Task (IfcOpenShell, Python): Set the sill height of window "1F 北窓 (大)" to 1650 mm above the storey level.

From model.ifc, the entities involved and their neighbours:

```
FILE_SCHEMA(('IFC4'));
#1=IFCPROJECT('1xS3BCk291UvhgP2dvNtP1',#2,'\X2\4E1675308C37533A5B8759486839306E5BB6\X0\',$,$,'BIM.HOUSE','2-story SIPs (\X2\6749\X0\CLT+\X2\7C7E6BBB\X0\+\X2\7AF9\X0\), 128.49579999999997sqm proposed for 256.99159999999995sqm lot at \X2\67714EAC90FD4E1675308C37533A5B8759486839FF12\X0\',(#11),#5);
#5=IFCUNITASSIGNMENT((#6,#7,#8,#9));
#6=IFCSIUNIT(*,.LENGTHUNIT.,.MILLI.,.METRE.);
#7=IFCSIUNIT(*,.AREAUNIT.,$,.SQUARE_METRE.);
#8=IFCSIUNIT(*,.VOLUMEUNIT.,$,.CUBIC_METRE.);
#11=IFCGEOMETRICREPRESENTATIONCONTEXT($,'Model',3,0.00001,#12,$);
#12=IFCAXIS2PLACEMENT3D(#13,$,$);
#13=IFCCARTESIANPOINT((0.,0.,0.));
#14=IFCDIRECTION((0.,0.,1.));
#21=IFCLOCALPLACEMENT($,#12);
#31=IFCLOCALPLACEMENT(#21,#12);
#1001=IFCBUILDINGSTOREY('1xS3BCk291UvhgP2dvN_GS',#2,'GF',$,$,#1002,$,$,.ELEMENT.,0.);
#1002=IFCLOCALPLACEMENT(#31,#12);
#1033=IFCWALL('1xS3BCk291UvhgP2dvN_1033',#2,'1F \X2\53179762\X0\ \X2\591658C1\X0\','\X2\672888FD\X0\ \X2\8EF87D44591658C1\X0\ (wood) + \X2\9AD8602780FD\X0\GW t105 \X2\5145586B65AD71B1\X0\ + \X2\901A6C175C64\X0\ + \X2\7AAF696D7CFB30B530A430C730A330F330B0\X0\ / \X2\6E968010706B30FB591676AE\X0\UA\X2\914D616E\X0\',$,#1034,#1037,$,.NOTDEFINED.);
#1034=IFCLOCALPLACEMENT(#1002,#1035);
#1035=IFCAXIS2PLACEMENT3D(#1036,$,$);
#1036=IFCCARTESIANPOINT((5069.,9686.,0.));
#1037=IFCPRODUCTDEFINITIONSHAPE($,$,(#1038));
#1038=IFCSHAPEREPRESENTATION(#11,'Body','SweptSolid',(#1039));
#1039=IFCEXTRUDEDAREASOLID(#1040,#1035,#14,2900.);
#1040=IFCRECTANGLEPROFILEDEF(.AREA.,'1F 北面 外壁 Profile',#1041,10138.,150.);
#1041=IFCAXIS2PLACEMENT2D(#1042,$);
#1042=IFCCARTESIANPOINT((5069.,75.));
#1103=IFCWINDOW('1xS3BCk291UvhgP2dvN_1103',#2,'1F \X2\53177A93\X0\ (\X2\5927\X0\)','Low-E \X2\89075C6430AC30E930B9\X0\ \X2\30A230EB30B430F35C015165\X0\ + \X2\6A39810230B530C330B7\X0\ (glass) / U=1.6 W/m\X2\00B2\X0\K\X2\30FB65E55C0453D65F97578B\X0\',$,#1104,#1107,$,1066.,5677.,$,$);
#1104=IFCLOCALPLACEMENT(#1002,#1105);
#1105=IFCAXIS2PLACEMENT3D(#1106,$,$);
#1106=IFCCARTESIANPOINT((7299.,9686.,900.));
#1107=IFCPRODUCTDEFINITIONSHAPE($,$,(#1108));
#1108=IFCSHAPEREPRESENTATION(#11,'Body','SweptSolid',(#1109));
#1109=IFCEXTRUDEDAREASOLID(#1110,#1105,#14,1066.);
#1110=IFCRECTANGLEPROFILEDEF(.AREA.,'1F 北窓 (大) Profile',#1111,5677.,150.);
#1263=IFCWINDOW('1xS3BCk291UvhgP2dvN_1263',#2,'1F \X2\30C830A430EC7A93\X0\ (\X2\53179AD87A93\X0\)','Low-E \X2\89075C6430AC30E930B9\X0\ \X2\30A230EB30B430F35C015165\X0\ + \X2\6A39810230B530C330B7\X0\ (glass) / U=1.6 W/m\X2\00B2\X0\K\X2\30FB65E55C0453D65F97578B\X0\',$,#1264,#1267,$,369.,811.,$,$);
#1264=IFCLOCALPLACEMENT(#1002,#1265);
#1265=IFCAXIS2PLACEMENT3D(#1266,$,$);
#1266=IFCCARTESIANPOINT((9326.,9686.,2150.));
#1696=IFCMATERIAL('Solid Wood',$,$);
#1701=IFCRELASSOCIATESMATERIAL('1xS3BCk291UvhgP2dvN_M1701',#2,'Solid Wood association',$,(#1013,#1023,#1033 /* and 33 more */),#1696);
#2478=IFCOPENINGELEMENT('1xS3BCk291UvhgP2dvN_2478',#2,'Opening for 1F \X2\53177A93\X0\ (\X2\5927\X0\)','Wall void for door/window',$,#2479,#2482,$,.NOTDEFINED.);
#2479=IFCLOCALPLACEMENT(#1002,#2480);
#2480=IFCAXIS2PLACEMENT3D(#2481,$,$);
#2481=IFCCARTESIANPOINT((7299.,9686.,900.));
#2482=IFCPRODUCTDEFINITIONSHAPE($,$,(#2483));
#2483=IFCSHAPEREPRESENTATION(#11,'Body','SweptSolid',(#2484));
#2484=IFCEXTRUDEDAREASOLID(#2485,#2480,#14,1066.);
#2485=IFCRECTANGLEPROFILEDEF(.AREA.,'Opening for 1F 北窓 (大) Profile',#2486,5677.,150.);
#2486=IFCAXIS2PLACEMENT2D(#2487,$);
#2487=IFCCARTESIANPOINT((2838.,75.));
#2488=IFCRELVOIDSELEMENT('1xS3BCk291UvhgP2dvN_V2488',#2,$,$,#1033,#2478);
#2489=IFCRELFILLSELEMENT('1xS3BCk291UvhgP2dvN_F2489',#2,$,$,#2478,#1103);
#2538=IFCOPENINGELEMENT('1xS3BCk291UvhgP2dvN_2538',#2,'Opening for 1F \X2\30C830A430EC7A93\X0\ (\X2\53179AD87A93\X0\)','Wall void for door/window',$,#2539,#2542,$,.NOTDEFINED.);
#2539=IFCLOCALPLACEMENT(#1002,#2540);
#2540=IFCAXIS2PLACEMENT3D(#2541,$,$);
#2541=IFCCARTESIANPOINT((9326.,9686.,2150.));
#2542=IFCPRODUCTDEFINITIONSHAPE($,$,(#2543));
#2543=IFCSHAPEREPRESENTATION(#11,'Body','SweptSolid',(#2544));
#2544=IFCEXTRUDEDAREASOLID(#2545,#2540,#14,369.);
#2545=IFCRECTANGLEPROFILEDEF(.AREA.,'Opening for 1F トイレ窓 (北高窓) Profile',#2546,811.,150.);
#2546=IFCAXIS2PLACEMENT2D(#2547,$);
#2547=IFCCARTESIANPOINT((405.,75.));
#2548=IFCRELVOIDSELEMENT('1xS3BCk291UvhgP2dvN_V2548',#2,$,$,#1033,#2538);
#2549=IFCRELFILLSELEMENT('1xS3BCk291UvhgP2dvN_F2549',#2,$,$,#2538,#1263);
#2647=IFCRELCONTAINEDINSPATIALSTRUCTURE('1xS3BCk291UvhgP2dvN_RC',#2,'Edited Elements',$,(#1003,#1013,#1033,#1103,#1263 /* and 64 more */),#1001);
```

```python
import numpy as np
import ifcopenshell
import ifcopenshell.api.geometry
import ifcopenshell.geom
import ifcopenshell.util.element
import ifcopenshell.util.placement
import ifcopenshell.util.shape
import ifcopenshell.util.unit

model = ifcopenshell.open("model.ifc")
unit_scale = ifcopenshell.util.unit.calculate_unit_scale(model)

window = model.by_id(1103)
opening = window.FillsVoids[0].RelatingOpeningElement
storey = ifcopenshell.util.element.get_container(window, ifc_class="IfcBuildingStorey")
level = ifcopenshell.util.placement.get_local_placement(storey.ObjectPlacement)[2, 3]

# The opening's origin need not be at the sill, so measure its lowest point.
shape = ifcopenshell.geom.create_shape(ifcopenshell.geom.settings(), opening)
bottom = ifcopenshell.util.shape.get_shape_bottom_elevation(shape, shape.geometry) / unit_scale
dz = level + 1.65 / unit_scale - bottom

shift = np.array([0.0, 0.0, dz])
# The window is not placed relative to its opening, so move both.
for product in (opening, window):
    matrix = ifcopenshell.util.placement.get_local_placement(product.ObjectPlacement)
    matrix[:3, 3] += shift
    ifcopenshell.api.geometry.edit_object_placement(model, product=product, matrix=matrix, is_si=False)

print(f"moved by {dz * unit_scale:+.3f} m")

model.write("model_v2.ifc")
```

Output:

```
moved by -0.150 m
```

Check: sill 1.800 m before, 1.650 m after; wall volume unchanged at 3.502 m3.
